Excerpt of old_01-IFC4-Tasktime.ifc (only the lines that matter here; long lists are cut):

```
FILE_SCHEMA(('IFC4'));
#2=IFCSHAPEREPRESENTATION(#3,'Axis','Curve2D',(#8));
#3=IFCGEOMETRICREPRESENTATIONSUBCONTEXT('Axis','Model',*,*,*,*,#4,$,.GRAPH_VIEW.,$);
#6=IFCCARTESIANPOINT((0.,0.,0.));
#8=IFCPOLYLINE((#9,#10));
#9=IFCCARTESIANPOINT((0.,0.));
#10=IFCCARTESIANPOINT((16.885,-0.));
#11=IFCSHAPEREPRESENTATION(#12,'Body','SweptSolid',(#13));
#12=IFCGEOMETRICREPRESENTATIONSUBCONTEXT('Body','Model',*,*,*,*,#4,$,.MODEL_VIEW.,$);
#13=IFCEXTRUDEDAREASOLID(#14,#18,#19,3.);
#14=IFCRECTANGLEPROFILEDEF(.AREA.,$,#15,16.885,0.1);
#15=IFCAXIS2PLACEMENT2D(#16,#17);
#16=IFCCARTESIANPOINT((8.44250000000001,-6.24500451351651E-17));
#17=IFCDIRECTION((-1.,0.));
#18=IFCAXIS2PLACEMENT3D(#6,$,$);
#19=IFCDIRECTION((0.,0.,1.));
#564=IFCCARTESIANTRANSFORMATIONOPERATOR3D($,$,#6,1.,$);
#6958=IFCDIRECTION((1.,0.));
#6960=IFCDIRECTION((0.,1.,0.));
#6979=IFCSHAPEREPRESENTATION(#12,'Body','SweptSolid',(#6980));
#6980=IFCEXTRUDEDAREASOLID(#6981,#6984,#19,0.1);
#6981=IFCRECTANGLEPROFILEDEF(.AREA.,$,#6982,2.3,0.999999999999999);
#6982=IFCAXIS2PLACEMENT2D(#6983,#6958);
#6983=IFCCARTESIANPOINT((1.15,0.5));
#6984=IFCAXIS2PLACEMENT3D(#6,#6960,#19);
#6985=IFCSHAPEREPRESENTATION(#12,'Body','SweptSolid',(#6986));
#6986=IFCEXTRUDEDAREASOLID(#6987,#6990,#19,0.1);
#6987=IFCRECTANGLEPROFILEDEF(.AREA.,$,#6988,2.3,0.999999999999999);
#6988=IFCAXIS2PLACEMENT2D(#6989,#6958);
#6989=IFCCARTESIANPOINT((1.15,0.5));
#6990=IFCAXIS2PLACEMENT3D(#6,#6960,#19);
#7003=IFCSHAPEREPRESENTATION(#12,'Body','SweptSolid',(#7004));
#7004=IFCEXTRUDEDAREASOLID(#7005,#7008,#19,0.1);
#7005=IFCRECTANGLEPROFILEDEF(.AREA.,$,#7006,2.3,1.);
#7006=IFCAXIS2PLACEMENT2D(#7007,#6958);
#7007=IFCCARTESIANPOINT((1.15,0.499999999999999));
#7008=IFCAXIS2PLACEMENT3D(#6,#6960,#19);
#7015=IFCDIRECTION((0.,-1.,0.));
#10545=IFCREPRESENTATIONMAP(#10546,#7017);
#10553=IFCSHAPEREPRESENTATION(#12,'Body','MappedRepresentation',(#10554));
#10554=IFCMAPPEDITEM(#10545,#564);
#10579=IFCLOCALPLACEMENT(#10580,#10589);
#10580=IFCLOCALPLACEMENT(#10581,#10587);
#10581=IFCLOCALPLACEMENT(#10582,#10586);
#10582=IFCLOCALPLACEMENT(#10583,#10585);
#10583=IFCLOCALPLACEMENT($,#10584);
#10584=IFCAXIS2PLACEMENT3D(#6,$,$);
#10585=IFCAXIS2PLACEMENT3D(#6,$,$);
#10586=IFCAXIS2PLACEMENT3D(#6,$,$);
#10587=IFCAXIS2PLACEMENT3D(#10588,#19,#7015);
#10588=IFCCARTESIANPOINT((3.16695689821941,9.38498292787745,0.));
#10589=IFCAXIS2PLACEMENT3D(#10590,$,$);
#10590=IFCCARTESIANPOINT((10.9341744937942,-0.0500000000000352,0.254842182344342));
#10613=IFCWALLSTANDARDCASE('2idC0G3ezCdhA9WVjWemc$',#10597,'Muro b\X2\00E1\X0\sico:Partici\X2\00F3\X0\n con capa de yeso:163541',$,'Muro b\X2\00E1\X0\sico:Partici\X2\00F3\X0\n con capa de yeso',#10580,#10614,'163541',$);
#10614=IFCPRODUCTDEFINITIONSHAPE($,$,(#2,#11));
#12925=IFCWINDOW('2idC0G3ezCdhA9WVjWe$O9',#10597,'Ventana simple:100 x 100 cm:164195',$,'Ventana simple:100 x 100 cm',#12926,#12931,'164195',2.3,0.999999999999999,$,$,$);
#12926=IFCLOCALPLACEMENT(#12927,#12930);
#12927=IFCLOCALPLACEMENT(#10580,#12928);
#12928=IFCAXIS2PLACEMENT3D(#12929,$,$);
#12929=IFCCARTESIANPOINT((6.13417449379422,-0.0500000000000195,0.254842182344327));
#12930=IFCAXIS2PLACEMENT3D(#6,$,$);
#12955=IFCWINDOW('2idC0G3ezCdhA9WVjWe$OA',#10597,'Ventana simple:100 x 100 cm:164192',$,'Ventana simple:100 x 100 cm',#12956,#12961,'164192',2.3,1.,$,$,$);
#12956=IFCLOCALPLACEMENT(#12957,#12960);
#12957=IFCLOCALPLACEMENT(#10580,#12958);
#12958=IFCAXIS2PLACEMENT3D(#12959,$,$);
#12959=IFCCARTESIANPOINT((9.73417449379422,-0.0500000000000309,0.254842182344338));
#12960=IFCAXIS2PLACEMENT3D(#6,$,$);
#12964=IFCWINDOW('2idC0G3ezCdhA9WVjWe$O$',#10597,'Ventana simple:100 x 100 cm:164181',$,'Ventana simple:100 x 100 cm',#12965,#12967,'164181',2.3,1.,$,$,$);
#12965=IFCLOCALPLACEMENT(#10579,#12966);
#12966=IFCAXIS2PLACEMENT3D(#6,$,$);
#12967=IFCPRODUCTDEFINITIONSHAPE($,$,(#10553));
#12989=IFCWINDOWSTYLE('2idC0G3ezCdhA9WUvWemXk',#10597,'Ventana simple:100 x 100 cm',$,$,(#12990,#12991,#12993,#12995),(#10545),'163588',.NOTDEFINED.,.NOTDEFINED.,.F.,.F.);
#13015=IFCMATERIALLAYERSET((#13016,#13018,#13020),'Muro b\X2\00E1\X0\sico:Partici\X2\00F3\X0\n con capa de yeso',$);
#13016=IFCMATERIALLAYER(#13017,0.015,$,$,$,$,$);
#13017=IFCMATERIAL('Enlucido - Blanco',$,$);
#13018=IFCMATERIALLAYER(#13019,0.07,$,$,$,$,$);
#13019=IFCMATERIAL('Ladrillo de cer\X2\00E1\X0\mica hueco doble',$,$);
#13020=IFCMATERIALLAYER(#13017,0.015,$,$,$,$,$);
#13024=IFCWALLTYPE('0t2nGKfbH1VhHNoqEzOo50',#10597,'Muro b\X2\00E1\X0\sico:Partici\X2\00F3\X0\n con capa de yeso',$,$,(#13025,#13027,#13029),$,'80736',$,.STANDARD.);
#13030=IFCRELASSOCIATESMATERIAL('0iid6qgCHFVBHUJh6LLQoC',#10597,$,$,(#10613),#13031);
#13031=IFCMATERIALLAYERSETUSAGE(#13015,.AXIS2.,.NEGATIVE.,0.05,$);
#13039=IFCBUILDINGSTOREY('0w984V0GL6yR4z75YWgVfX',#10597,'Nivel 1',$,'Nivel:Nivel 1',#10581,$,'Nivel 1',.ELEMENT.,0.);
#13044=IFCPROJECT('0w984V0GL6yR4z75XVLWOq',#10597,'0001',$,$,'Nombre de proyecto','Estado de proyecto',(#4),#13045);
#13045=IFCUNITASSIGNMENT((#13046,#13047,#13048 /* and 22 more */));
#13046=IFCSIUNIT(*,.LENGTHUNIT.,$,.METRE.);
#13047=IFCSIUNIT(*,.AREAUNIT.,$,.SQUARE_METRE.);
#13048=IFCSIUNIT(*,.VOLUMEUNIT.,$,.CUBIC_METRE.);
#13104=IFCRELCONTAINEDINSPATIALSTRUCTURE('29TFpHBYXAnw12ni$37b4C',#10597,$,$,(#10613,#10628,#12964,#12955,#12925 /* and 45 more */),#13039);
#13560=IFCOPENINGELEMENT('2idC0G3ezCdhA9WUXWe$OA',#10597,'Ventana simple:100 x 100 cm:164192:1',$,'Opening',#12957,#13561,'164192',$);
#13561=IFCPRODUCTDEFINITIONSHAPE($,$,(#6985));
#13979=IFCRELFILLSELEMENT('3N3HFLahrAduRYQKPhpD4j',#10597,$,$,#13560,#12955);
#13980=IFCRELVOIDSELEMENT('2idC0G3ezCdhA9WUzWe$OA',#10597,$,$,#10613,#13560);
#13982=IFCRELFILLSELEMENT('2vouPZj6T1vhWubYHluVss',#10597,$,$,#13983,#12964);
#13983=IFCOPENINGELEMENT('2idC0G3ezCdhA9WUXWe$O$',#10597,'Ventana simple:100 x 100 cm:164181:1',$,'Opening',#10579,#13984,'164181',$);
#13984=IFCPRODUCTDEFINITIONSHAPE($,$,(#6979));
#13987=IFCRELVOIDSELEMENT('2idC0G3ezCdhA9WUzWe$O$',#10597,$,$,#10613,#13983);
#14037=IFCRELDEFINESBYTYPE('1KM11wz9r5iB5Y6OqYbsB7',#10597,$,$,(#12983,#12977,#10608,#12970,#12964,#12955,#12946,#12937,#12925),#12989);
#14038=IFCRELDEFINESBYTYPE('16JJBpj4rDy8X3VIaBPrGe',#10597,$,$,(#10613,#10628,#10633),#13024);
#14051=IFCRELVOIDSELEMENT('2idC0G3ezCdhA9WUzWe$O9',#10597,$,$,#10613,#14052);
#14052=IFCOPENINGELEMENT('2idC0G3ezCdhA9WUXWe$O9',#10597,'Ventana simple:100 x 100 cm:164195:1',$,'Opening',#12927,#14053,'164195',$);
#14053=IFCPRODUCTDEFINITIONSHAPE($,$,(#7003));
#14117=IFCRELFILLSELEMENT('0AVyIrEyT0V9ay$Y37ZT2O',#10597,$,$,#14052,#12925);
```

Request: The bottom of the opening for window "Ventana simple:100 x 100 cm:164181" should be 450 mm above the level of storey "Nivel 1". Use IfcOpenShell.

```python
import numpy as np
import ifcopenshell
import ifcopenshell.api.geometry
import ifcopenshell.geom
import ifcopenshell.util.element
import ifcopenshell.util.placement
import ifcopenshell.util.shape
import ifcopenshell.util.unit

model = ifcopenshell.open("old_01-IFC4-Tasktime.ifc")
unit_scale = ifcopenshell.util.unit.calculate_unit_scale(model)

window = model.by_guid("2idC0G3ezCdhA9WVjWe$O$")
opening = window.FillsVoids[0].RelatingOpeningElement
storey = ifcopenshell.util.element.get_container(window, ifc_class="IfcBuildingStorey")
level = ifcopenshell.util.placement.get_local_placement(storey.ObjectPlacement)[2, 3]

# The opening's origin need not be at the sill, so measure its lowest point.
shape = ifcopenshell.geom.create_shape(ifcopenshell.geom.settings(), opening)
bottom = ifcopenshell.util.shape.get_shape_bottom_elevation(shape, shape.geometry) / unit_scale
dz = level + 0.45 - bottom

shift = np.array([0.0, 0.0, dz])
# The window is placed relative to its opening, so it follows when the opening moves.
matrix = ifcopenshell.util.placement.get_local_placement(opening.ObjectPlacement)
matrix[:3, 3] += shift
ifcopenshell.api.geometry.edit_object_placement(
    model, product=opening, matrix=matrix, is_si=False, should_transform_children=True
)

print(f"moved by {dz * unit_scale:+.3f} m")

model.write("old_01-IFC4-Tasktime_edited.ifc")
```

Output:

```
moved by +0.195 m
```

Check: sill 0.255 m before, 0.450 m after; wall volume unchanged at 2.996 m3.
